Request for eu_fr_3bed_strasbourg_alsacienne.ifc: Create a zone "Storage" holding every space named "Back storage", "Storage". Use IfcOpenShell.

First a look at what the model holds.

```python
import ifcopenshell

model = ifcopenshell.open("eu_fr_3bed_strasbourg_alsacienne.ifc")
print(model.schema)
seen = {}
for space in model.by_type("IfcSpace"):
    seen[space.LongName] = seen.get(space.LongName, 0) + 1
for name, count in sorted(seen.items(), key=str):
    print(count, "x", name)
print("zones:", [z.Name for z in model.by_type("IfcZone")][:20])
```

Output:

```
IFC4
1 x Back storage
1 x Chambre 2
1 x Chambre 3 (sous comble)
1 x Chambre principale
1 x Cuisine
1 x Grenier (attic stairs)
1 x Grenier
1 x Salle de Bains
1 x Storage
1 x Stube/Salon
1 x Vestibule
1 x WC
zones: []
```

```python
import ifcopenshell
import ifcopenshell.api.group
import ifcopenshell.api.root

model = ifcopenshell.open("eu_fr_3bed_strasbourg_alsacienne.ifc")

names = {"Back storage", "Storage"}
spaces = [s for s in model.by_type("IfcSpace") if s.LongName in names]

zone = ifcopenshell.api.root.create_entity(model, ifc_class="IfcZone", name="Storage")
ifcopenshell.api.group.assign_group(model, products=spaces, group=zone)
print(len(spaces), "spaces in", zone.Name)

model.write("eu_fr_3bed_strasbourg_alsacienne-out.ifc")
```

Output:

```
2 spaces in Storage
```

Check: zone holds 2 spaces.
